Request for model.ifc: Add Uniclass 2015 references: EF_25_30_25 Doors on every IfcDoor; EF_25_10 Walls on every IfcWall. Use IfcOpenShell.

First a look at what the model holds.

```python
import ifcopenshell

model = ifcopenshell.open("model.ifc")
print(model.schema)
print("classifications:", [c.Name for c in model.by_type("IfcClassification")])
for ifc_class in ("IfcDoor", "IfcRoof", "IfcStair", "IfcWall", "IfcWindow"):
    print(ifc_class, len(model.by_type(ifc_class)))
```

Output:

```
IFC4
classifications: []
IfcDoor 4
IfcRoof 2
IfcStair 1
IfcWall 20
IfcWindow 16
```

```python
import ifcopenshell
import ifcopenshell.api.classification

model = ifcopenshell.open("model.ifc")

system = ifcopenshell.api.classification.add_classification(model, classification="Uniclass 2015")

codes = {
    "IfcDoor": ("EF_25_30_25", "Doors"),
    "IfcWall": ("EF_25_10", "Walls"),
}
for ifc_class, (code, name) in codes.items():
    products = model.by_type(ifc_class)
    ifcopenshell.api.classification.add_reference(
        model, products=products, classification=system, identification=code, name=name
    )
    print(code, len(products))

model.write("model_updated.ifc")
```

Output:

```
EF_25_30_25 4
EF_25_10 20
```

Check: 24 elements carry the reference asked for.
